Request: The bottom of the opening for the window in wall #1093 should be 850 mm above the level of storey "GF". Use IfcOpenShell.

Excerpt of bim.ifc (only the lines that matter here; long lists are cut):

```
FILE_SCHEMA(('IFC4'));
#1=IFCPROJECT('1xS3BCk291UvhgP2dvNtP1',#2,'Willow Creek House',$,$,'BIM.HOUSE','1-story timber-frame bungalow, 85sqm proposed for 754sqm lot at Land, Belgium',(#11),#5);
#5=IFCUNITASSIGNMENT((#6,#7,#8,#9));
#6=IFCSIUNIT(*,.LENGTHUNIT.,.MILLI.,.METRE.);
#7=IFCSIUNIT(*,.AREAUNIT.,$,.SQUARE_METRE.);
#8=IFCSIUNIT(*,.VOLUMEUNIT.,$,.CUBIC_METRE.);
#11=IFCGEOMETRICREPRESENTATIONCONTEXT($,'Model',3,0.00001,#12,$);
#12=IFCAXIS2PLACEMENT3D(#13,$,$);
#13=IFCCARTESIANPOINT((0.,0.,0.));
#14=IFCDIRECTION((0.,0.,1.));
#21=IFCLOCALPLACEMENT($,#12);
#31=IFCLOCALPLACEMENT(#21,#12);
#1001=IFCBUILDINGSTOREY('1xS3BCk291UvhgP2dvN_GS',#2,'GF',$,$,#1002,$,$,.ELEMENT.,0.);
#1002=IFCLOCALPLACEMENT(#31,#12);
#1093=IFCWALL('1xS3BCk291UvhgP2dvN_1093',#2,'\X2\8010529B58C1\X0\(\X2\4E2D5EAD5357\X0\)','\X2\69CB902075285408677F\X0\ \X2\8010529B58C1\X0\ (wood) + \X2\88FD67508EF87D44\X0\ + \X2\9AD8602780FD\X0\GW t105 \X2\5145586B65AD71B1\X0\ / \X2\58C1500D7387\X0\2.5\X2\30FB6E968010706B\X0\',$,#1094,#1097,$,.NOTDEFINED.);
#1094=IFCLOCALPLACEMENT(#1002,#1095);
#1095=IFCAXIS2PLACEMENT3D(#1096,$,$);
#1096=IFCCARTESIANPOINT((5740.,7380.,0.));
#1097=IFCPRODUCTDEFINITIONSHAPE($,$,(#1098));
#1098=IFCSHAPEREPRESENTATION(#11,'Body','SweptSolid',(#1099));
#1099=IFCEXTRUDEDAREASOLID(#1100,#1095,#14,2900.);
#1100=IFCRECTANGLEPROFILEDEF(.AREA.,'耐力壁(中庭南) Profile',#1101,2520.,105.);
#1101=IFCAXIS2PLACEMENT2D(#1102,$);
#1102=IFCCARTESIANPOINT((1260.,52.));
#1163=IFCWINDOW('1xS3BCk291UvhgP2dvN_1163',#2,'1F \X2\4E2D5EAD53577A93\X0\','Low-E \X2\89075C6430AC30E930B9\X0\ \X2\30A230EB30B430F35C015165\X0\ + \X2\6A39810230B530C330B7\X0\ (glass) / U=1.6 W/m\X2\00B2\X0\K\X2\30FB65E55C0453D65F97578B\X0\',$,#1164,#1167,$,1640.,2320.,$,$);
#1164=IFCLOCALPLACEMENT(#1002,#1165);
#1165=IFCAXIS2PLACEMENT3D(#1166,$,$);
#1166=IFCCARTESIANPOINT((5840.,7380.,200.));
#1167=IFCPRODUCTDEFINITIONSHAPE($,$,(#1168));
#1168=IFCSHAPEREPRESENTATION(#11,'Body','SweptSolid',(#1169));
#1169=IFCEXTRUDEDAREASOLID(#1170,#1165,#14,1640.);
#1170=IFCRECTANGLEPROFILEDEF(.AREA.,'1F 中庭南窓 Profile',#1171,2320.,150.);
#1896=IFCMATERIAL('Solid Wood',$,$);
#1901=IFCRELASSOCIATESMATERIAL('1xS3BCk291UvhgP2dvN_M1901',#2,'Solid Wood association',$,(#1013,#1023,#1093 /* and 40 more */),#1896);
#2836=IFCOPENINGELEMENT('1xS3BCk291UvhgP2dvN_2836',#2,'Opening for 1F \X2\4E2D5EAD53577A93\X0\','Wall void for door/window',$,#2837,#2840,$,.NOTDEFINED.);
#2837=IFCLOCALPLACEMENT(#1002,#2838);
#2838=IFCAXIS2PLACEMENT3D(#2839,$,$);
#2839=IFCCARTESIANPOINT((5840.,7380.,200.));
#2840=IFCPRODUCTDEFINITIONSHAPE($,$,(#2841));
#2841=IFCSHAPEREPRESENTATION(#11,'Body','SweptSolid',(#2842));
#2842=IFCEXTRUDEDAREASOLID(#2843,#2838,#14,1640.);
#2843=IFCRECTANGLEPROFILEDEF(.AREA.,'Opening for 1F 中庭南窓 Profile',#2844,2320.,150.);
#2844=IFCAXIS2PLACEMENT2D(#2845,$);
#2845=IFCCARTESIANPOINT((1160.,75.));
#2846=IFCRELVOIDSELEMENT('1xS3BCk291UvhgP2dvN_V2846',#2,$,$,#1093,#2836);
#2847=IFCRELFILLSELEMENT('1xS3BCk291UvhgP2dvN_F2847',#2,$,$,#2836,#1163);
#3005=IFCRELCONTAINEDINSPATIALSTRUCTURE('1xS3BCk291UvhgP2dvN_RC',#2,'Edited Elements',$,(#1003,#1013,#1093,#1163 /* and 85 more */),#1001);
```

```python
import numpy as np
import ifcopenshell
import ifcopenshell.api.geometry
import ifcopenshell.geom
import ifcopenshell.util.element
import ifcopenshell.util.placement
import ifcopenshell.util.shape
import ifcopenshell.util.unit

model = ifcopenshell.open("bim.ifc")
unit_scale = ifcopenshell.util.unit.calculate_unit_scale(model)

window = model.by_guid("1xS3BCk291UvhgP2dvN_1163")
opening = window.FillsVoids[0].RelatingOpeningElement
storey = ifcopenshell.util.element.get_container(window, ifc_class="IfcBuildingStorey")
level = ifcopenshell.util.placement.get_local_placement(storey.ObjectPlacement)[2, 3]

# The opening's origin need not be at the sill, so measure its lowest point.
shape = ifcopenshell.geom.create_shape(ifcopenshell.geom.settings(), opening)
bottom = ifcopenshell.util.shape.get_shape_bottom_elevation(shape, shape.geometry) / unit_scale
dz = level + 0.85 / unit_scale - bottom

shift = np.array([0.0, 0.0, dz])
# The window is not placed relative to its opening, so move both.
for product in (opening, window):
    matrix = ifcopenshell.util.placement.get_local_placement(product.ObjectPlacement)
    matrix[:3, 3] += shift
    ifcopenshell.api.geometry.edit_object_placement(model, product=product, matrix=matrix, is_si=False)

print(f"moved by {dz * unit_scale:+.3f} m")

model.write("bim_updated.ifc")
```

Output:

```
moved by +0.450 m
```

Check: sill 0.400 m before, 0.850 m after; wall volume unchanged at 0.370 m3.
